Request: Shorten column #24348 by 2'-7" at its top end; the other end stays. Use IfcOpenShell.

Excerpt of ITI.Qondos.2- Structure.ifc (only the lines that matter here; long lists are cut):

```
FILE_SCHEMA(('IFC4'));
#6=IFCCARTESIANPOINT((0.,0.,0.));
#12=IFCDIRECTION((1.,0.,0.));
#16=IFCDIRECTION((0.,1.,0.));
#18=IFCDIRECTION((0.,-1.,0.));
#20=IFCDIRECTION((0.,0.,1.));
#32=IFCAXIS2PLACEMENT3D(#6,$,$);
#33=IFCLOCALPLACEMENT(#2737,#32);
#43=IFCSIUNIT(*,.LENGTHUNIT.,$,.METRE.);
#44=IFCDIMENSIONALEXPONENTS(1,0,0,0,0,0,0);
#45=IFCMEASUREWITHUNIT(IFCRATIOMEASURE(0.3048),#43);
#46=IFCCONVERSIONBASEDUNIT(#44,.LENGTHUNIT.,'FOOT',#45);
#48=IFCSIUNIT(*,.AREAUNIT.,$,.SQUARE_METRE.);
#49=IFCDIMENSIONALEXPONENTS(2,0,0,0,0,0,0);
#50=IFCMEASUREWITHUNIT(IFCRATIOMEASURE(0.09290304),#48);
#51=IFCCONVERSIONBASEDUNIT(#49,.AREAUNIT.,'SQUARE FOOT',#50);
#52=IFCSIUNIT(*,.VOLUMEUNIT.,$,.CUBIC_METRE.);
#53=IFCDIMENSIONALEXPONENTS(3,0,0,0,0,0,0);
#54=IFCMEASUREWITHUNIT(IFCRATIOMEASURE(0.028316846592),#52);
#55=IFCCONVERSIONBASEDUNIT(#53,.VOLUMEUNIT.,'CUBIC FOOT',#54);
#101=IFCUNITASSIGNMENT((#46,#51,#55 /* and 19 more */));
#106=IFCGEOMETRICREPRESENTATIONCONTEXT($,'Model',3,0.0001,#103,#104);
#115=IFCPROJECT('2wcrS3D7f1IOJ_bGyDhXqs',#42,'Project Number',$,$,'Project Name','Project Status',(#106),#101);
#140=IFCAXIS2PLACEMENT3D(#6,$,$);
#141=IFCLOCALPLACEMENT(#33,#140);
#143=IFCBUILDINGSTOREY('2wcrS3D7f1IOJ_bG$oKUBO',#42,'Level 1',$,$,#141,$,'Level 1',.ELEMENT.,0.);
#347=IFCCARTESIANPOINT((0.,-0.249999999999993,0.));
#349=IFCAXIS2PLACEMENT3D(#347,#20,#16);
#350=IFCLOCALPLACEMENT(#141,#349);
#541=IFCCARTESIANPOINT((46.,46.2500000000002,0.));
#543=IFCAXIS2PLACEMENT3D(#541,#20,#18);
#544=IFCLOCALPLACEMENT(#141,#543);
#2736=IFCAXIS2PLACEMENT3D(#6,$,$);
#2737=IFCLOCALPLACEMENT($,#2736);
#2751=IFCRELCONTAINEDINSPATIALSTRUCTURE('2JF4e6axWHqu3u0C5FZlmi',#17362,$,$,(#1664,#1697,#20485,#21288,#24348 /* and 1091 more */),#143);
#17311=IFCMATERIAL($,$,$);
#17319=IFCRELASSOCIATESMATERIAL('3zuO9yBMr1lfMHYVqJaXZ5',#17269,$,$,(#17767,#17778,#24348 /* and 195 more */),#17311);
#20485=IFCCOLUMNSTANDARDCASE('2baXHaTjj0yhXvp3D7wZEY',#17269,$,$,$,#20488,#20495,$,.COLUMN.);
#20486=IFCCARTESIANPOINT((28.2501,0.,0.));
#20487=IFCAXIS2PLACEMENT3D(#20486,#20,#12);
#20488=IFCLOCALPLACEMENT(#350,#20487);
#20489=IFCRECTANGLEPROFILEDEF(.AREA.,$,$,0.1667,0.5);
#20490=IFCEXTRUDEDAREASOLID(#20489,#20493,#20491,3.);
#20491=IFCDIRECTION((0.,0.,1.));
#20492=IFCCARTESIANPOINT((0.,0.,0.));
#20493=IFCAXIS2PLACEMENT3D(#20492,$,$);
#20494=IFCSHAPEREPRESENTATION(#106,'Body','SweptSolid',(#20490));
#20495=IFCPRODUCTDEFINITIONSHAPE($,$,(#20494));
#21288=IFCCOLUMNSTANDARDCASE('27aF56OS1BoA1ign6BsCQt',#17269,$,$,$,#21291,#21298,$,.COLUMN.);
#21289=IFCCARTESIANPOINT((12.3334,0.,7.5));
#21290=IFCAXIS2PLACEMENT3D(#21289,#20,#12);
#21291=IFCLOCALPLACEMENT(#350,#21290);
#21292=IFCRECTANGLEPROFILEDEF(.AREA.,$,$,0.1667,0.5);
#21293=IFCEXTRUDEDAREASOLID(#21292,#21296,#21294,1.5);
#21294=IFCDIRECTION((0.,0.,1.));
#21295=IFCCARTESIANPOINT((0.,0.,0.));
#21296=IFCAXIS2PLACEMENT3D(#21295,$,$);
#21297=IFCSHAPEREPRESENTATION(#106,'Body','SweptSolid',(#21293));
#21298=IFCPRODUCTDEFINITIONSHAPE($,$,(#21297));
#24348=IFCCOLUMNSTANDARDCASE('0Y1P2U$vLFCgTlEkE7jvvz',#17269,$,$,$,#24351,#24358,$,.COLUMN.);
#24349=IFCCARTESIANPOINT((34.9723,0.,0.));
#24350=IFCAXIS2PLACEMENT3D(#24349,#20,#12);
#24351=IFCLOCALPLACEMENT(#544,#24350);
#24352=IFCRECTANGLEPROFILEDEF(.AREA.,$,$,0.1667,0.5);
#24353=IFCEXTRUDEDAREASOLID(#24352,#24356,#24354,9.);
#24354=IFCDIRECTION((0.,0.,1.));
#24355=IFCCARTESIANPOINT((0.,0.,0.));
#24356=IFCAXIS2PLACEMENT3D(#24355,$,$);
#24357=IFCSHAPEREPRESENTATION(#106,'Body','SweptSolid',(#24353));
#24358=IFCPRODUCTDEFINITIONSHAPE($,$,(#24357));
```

```python
import ifcopenshell
import ifcopenshell.util.unit

model = ifcopenshell.open("ITI.Qondos.2- Structure.ifc")
unit_scale = ifcopenshell.util.unit.calculate_unit_scale(model)

member = model.by_id(24348)
change = -31 * 0.0254 / unit_scale

# The extrusion runs towards the end named, so only its depth changes.
body = next(r for r in member.Representation.Representations if r.RepresentationIdentifier == "Body")
solid = body.Items[0]
old_length = solid.Depth
solid.Depth += change

print(f"length {old_length:g} -> {solid.Depth:g}")

model.write("ITI.Qondos.2- Structure_v2.ifc")
```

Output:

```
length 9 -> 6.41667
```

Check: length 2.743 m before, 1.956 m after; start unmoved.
